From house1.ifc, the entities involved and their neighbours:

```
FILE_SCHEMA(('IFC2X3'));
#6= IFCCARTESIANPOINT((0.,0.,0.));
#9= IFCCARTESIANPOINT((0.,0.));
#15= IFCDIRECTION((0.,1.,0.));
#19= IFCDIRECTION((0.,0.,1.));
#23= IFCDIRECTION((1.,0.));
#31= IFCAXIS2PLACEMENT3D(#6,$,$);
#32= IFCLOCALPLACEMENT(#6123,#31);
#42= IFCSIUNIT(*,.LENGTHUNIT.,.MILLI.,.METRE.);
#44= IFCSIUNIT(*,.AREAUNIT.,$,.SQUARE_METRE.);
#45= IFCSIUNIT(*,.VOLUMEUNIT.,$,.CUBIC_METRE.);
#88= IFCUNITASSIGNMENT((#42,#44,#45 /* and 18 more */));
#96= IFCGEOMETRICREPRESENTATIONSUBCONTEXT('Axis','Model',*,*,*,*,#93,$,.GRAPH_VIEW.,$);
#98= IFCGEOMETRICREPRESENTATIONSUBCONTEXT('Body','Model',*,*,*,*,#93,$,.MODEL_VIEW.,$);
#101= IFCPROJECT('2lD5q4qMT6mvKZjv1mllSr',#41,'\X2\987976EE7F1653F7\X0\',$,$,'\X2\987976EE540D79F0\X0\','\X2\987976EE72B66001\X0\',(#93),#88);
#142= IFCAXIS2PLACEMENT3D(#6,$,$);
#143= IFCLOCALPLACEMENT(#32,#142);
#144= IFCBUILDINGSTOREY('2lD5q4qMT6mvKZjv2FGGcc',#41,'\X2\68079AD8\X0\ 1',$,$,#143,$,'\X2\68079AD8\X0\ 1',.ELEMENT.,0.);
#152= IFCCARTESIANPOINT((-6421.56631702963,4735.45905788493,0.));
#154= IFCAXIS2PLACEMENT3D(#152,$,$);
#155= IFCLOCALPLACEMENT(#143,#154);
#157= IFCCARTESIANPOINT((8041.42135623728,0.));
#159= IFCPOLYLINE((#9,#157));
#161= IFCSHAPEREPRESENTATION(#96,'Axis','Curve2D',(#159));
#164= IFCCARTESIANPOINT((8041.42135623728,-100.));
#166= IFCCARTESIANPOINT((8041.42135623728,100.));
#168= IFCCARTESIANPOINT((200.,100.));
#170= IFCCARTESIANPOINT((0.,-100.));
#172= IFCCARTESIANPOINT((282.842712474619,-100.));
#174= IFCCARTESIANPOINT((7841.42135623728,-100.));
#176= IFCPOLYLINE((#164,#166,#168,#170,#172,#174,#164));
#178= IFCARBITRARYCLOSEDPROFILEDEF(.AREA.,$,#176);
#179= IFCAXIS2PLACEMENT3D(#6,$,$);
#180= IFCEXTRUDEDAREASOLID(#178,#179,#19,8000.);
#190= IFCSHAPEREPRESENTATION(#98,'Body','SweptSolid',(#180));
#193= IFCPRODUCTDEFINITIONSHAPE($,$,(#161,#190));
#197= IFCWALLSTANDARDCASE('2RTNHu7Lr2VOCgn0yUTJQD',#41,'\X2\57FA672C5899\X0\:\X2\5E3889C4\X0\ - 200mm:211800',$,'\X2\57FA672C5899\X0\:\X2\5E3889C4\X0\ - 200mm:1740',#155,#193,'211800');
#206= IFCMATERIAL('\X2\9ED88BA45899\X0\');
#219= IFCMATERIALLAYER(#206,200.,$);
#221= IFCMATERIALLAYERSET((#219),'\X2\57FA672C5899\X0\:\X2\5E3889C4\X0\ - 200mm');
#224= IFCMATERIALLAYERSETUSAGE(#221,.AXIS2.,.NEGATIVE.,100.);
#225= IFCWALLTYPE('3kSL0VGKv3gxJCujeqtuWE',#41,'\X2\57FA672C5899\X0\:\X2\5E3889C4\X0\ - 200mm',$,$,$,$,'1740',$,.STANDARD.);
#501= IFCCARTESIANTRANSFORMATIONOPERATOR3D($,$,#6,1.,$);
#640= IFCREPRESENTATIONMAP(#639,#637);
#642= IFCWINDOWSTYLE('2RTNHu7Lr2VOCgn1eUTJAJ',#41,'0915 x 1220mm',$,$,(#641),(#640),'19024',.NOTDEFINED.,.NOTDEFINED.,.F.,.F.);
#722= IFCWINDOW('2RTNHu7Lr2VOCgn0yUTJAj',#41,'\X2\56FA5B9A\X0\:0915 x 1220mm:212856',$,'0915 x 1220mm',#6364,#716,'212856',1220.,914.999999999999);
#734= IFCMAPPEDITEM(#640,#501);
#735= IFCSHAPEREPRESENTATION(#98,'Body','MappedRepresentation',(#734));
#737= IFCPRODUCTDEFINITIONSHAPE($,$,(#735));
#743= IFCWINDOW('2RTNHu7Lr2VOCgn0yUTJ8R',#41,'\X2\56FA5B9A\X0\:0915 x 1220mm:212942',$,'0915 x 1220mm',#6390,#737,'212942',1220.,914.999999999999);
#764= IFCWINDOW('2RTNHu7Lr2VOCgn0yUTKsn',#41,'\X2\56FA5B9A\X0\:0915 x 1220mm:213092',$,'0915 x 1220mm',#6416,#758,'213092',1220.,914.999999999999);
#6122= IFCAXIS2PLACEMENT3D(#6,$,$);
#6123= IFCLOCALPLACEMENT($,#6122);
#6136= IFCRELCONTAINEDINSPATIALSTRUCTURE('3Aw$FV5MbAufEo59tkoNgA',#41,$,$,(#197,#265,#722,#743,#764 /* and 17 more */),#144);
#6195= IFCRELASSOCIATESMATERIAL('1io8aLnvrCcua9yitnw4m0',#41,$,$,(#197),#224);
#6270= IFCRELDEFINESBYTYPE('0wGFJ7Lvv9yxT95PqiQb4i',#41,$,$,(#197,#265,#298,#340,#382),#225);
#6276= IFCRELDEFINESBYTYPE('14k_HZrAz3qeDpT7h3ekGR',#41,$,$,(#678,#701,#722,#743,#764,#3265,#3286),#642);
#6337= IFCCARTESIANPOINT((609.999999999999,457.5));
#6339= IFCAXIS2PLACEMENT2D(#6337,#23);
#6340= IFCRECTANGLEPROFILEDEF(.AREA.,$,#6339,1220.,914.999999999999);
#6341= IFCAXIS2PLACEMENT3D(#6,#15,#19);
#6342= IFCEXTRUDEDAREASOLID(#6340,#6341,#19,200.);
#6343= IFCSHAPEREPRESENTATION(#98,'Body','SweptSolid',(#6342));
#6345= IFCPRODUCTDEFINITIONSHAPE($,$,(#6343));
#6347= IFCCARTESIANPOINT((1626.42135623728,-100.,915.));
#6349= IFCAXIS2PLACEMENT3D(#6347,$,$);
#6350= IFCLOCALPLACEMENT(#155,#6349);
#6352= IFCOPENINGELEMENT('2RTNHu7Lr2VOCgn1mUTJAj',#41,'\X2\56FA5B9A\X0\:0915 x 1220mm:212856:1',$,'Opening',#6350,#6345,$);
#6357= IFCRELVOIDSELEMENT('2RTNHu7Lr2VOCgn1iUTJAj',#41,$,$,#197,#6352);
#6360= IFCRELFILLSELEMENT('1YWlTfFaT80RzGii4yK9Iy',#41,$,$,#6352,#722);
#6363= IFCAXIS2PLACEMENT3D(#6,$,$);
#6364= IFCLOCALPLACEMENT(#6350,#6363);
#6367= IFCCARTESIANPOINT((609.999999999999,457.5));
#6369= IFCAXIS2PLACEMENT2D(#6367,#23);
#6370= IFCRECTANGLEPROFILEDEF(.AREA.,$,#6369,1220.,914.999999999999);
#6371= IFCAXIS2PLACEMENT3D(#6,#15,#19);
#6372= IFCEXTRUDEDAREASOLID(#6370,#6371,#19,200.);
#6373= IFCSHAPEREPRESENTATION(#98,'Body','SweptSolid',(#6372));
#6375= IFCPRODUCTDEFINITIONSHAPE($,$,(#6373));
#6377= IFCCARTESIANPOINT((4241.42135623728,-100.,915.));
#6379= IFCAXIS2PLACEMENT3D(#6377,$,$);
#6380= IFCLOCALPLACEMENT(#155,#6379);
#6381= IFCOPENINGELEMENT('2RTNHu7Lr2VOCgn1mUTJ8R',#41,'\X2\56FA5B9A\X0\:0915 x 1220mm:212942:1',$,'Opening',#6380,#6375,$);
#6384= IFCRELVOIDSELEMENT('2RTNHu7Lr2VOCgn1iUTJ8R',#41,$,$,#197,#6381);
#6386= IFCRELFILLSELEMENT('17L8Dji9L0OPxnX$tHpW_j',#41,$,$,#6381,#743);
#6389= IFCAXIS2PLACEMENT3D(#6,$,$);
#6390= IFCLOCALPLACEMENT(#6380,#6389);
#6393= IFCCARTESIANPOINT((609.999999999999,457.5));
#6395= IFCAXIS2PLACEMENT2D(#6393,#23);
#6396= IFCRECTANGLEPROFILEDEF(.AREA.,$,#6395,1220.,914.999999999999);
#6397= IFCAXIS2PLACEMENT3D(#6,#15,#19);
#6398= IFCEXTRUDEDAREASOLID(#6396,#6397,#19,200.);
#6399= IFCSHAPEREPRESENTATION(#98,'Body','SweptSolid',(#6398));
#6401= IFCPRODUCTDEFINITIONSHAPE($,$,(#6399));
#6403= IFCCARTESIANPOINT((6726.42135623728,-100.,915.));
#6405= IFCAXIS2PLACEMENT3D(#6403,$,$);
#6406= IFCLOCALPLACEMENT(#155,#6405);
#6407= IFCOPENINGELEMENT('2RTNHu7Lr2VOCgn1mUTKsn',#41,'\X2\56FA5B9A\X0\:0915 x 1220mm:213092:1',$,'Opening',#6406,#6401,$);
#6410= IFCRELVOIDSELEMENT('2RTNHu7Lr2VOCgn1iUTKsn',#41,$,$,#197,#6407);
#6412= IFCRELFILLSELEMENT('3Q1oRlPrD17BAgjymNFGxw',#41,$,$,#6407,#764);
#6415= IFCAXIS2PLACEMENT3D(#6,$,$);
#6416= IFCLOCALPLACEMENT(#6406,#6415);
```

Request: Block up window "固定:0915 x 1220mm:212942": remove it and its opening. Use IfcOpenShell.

```python
import ifcopenshell
import ifcopenshell.api.feature
import ifcopenshell.api.root
import ifcopenshell.geom
import ifcopenshell.util.shape

model = ifcopenshell.open("house1.ifc")
settings = ifcopenshell.geom.settings()


def volume(element):
    """Net volume in cubic metres, openings subtracted."""
    shape = ifcopenshell.geom.create_shape(settings, element)
    return ifcopenshell.util.shape.get_volume(shape.geometry)


window = model.by_guid("2RTNHu7Lr2VOCgn0yUTJ8R")
opening = window.FillsVoids[0].RelatingOpeningElement
wall = opening.VoidsElements[0].RelatingBuildingElement
before = volume(wall)

ifcopenshell.api.root.remove_product(model, product=window)
ifcopenshell.api.feature.remove_feature(model, feature=opening)

after = volume(wall)

print(f"wall volume {before:.3f} -> {after:.3f} m3")

model.write("house1_updated.ifc")
```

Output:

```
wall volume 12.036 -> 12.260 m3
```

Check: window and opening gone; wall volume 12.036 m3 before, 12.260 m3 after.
